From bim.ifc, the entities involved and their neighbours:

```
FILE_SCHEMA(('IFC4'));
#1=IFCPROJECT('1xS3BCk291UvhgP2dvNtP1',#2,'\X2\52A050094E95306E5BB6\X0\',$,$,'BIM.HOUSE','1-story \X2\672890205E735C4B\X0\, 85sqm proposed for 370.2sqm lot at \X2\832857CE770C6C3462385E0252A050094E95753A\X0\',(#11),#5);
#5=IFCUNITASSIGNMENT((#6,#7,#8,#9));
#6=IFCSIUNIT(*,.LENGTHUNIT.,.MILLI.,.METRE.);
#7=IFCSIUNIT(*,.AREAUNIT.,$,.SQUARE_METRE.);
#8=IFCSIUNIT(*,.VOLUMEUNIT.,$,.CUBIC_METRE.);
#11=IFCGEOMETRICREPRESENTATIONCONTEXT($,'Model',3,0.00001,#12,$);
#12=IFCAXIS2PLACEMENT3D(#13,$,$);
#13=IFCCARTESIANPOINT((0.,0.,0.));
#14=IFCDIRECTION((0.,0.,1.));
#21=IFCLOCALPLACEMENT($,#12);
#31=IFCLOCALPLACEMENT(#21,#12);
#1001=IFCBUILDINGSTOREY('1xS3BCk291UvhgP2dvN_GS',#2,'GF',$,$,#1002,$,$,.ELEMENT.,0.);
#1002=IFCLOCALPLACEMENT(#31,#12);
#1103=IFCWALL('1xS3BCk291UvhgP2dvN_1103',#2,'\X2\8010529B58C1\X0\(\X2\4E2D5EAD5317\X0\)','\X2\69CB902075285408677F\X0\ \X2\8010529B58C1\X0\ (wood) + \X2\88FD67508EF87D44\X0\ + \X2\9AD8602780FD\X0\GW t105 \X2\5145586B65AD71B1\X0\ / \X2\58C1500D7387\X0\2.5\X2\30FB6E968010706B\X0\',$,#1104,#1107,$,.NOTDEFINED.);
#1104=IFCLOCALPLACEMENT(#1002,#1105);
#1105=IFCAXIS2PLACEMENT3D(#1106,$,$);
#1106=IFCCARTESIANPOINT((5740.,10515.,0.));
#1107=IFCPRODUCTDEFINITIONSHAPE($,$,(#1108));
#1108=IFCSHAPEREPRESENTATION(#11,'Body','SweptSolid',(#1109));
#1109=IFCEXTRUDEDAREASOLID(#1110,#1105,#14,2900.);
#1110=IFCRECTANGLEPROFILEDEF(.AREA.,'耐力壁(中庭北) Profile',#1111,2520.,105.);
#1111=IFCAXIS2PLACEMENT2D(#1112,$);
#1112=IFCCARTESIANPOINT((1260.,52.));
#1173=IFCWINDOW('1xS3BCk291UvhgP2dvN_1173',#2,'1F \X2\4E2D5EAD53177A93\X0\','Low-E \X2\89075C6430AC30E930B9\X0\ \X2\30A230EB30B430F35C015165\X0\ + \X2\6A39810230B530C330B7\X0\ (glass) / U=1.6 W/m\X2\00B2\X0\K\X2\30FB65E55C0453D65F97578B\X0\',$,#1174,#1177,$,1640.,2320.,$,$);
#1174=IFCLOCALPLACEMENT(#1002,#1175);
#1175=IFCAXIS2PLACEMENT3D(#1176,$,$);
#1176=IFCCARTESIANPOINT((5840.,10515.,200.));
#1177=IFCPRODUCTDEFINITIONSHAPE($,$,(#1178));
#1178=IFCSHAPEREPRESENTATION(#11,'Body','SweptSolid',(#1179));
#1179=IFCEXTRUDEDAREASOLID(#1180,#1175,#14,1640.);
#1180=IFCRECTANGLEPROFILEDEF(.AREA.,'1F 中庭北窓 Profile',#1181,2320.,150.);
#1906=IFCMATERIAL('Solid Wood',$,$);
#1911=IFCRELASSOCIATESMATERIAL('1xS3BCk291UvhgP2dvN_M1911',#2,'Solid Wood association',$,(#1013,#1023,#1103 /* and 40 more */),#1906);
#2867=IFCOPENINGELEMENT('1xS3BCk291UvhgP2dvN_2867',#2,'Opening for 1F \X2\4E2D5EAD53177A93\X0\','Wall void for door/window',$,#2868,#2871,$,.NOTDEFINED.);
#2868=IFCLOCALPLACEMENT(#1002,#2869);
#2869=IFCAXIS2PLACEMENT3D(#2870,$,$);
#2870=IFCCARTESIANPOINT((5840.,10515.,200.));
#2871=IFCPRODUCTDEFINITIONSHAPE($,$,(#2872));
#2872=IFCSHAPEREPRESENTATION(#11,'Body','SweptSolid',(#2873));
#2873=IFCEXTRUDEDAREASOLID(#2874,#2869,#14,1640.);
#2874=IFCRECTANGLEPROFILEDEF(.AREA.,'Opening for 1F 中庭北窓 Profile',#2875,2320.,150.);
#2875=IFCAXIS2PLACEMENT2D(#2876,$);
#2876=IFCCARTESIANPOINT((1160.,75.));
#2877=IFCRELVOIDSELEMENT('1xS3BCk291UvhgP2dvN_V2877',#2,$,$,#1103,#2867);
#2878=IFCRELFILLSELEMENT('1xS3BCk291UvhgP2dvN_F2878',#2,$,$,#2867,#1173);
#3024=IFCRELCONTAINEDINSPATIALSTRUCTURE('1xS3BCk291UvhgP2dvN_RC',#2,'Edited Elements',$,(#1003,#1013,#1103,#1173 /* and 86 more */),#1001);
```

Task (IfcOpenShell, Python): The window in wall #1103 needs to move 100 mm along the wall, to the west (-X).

```python
import ifcopenshell
import ifcopenshell.api.geometry
import ifcopenshell.util.placement
import ifcopenshell.util.unit

model = ifcopenshell.open("bim.ifc")
unit_scale = ifcopenshell.util.unit.calculate_unit_scale(model)

window = model.by_id(1173)
opening = window.FillsVoids[0].RelatingOpeningElement
wall = opening.VoidsElements[0].RelatingBuildingElement

wall_matrix = ifcopenshell.util.placement.get_local_placement(wall.ObjectPlacement)
shift = wall_matrix[:3, 0] * -0.1 / unit_scale
before = ifcopenshell.util.placement.get_local_placement(window.ObjectPlacement)[:3, 3].copy()

# The window is not placed relative to its opening, so move both.
for product in (opening, window):
    matrix = ifcopenshell.util.placement.get_local_placement(product.ObjectPlacement)
    matrix[:3, 3] += shift
    ifcopenshell.api.geometry.edit_object_placement(model, product=product, matrix=matrix, is_si=False)

after = ifcopenshell.util.placement.get_local_placement(window.ObjectPlacement)[:3, 3]
print("window moved by", (after - before).round(3) + 0.0)

model.write("bim-out.ifc")
```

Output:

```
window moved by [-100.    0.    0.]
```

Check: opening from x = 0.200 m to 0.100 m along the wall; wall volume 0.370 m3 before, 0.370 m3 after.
